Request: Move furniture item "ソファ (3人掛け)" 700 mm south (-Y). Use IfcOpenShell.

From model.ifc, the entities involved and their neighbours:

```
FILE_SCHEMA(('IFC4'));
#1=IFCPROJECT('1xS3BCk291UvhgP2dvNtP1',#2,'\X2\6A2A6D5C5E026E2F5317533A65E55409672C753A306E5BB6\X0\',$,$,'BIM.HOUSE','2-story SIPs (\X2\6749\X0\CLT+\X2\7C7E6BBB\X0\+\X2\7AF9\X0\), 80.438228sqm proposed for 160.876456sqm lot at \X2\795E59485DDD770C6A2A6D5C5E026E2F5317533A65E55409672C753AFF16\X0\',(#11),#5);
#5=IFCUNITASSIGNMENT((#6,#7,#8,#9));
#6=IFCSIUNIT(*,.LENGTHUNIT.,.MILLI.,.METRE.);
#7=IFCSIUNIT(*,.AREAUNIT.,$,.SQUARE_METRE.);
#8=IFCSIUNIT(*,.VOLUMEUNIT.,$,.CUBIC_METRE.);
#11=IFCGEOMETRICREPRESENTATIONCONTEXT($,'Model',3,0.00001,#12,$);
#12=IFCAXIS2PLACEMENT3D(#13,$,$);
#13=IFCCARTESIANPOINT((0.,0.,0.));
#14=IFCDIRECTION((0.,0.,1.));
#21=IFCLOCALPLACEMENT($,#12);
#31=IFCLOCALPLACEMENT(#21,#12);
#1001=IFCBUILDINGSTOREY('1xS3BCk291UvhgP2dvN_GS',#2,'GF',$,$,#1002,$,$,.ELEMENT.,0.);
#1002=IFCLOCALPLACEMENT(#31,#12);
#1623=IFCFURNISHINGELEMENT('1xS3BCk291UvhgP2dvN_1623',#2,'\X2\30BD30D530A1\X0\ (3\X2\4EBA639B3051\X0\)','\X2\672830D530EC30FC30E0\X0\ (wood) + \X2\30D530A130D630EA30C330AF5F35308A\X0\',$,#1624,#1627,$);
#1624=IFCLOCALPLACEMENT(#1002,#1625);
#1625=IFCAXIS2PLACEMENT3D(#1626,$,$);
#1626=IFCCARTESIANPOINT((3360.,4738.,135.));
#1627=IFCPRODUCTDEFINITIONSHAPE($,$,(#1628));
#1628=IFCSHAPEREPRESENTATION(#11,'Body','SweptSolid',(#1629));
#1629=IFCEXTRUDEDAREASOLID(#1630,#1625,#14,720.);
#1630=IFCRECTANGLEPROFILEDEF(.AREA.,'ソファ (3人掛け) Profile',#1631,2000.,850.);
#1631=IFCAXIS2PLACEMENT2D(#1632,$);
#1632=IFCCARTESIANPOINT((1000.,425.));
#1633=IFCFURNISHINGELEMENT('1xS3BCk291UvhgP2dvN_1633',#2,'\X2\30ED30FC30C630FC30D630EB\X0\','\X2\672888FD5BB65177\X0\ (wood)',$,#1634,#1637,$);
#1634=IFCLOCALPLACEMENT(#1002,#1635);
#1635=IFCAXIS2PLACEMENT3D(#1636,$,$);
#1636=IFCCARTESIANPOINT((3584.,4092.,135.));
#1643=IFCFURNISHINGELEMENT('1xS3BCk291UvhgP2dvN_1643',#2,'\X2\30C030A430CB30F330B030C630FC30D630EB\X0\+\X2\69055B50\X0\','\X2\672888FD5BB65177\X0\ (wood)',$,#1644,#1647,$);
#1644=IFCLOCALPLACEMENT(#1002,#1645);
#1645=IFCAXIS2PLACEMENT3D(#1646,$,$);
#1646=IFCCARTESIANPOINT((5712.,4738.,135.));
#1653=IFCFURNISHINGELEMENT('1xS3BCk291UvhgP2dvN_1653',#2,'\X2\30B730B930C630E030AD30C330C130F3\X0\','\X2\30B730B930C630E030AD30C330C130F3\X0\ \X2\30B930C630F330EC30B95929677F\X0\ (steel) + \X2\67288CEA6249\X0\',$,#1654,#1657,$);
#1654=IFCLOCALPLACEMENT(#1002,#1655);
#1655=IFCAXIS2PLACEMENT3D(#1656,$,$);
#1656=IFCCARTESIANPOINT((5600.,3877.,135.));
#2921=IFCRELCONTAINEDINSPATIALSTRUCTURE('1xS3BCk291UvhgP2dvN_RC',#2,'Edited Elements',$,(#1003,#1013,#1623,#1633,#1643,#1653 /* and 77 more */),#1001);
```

```python
import ifcopenshell
import ifcopenshell.api.geometry
import ifcopenshell.util.placement

model = ifcopenshell.open("model.ifc")

item = model.by_guid("1xS3BCk291UvhgP2dvN_1623")
matrix = ifcopenshell.util.placement.get_local_placement(item.ObjectPlacement)
matrix[1, 3] -= 700.0
ifcopenshell.api.geometry.edit_object_placement(model, product=item, matrix=matrix, is_si=False)

print(ifcopenshell.util.placement.get_local_placement(item.ObjectPlacement).round(3) + 0.0)

model.write("model_edited.ifc")
```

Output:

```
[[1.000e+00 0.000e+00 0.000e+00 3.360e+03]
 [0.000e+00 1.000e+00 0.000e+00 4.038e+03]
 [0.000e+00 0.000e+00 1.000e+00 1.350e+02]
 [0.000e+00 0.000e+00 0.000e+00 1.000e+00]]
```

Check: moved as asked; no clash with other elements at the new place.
